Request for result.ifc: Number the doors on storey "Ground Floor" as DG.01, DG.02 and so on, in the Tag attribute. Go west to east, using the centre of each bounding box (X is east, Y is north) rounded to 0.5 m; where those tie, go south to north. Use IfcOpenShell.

First a look at what the model holds.

```python
import ifcopenshell
import ifcopenshell.util.element
import ifcopenshell.util.placement

model = ifcopenshell.open("result.ifc")
print(model.schema)
storey = next(s for s in model.by_type("IfcBuildingStorey") if s.Name == "Ground Floor")
doors = [e for e in ifcopenshell.util.element.get_decomposition(storey) if e.is_a("IfcDoor")]
for e in sorted(doors, key=lambda e: e.id()):
    origin = ifcopenshell.util.placement.get_local_placement(e.ObjectPlacement)[:3, 3]
    print(e.id(), e.Tag, e.Name, origin.round(2) + 0.0, sep=" | ")
```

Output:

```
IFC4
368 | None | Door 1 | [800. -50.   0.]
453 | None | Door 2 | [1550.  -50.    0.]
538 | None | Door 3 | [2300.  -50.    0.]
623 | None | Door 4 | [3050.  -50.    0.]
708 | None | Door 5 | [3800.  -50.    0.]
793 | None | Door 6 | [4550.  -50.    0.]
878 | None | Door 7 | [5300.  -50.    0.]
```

```python
import ifcopenshell
import ifcopenshell.geom
import ifcopenshell.util.element
import ifcopenshell.util.shape

model = ifcopenshell.open("result.ifc")
settings = ifcopenshell.geom.settings()
settings.set("use-world-coords", True)


def centre(element):
    shape = ifcopenshell.geom.create_shape(settings, element)
    return ifcopenshell.util.shape.get_bbox_centroid(shape.geometry)


storey = next(s for s in model.by_type("IfcBuildingStorey") if s.Name == "Ground Floor")
doors = [e for e in ifcopenshell.util.element.get_decomposition(storey) if e.is_a("IfcDoor")]

# Insertion points can sit at a corner or the storey origin, so sort by the geometry (in metres).
centres = {e: centre(e) for e in doors}
doors.sort(key=lambda e: (round(centres[e][0] / 0.5), centres[e][1]))

for i, e in enumerate(doors, start=1):
    number = f"DG.{i:02d}"
    e.Tag = number
    print(e.id(), number)

model.write("result_v2.ifc")
```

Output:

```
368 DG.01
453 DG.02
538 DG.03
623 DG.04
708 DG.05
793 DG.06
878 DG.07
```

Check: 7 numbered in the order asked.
